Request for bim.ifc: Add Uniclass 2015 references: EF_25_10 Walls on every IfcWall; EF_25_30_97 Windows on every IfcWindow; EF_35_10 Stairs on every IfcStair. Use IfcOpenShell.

First a look at what the model holds.

```python
import ifcopenshell

model = ifcopenshell.open("bim.ifc")
print(model.schema)
print("classifications:", [c.Name for c in model.by_type("IfcClassification")])
for ifc_class in ("IfcDoor", "IfcRoof", "IfcStair", "IfcWall", "IfcWindow"):
    print(ifc_class, len(model.by_type(ifc_class)))
```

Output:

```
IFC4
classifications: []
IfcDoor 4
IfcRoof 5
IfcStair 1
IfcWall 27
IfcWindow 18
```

```python
import ifcopenshell
import ifcopenshell.api.classification

model = ifcopenshell.open("bim.ifc")

system = ifcopenshell.api.classification.add_classification(model, classification="Uniclass 2015")

codes = {
    "IfcWall": ("EF_25_10", "Walls"),
    "IfcWindow": ("EF_25_30_97", "Windows"),
    "IfcStair": ("EF_35_10", "Stairs"),
}
for ifc_class, (code, name) in codes.items():
    products = model.by_type(ifc_class)
    ifcopenshell.api.classification.add_reference(
        model, products=products, classification=system, identification=code, name=name
    )
    print(code, len(products))

model.write("bim-out.ifc")
```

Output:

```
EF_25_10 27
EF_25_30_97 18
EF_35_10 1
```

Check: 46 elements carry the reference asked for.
